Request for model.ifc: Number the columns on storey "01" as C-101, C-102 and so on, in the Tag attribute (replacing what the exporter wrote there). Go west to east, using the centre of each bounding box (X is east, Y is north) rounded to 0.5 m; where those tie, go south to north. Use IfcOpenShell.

First a look at what the model holds.

```python
import ifcopenshell
import ifcopenshell.util.element
import ifcopenshell.util.placement

model = ifcopenshell.open("model.ifc")
print(model.schema)
storey = next(s for s in model.by_type("IfcBuildingStorey") if s.Name == "01")
columns = [e for e in ifcopenshell.util.element.get_decomposition(storey) if e.is_a("IfcColumn")]
for e in sorted(columns, key=lambda e: e.id()):
    origin = ifcopenshell.util.placement.get_local_placement(e.ObjectPlacement)[:3, 3]
    print(e.id(), e.Tag, e.Name, origin.round(2) + 0.0, sep=" | ")
```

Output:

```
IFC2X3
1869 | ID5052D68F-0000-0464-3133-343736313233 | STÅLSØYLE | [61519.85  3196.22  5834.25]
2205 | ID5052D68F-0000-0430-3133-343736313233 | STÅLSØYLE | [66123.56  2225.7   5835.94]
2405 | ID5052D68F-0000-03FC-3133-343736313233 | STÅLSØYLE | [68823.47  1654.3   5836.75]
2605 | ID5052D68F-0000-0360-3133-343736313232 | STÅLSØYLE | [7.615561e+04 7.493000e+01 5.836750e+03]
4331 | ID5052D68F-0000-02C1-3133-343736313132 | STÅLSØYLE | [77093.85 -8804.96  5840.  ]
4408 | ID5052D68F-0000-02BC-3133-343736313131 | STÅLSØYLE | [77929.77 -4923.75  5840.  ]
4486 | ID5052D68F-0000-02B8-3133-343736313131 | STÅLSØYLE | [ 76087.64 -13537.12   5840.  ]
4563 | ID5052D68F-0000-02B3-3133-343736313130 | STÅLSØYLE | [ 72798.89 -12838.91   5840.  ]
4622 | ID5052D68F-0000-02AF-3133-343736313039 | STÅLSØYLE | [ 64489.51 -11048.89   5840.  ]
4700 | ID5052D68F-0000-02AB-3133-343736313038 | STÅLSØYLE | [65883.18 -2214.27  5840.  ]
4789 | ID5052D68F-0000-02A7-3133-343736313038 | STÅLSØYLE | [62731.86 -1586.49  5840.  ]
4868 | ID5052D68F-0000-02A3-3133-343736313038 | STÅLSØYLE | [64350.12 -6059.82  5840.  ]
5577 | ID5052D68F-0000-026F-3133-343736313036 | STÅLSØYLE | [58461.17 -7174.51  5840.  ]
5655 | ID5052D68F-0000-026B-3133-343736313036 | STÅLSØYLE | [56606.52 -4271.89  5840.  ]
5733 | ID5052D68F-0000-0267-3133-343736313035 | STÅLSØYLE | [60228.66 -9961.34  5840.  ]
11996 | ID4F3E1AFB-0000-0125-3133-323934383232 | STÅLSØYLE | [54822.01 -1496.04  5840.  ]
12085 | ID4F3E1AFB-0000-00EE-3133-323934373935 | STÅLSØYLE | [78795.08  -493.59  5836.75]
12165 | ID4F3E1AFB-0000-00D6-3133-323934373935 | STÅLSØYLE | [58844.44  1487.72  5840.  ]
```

```python
import ifcopenshell
import ifcopenshell.geom
import ifcopenshell.util.element
import ifcopenshell.util.shape

model = ifcopenshell.open("model.ifc")
settings = ifcopenshell.geom.settings()
settings.set("use-world-coords", True)


def centre(element):
    shape = ifcopenshell.geom.create_shape(settings, element)
    return ifcopenshell.util.shape.get_bbox_centroid(shape.geometry)


storey = next(s for s in model.by_type("IfcBuildingStorey") if s.Name == "01")
columns = [e for e in ifcopenshell.util.element.get_decomposition(storey) if e.is_a("IfcColumn")]

# Insertion points can sit at a corner or the storey origin, so sort by the geometry (in metres).
centres = {e: centre(e) for e in columns}
columns.sort(key=lambda e: (round(centres[e][0] / 0.5), centres[e][1]))

for i, e in enumerate(columns, start=1):
    number = f"C-1{i:02d}"
    e.Tag = number
    print(e.id(), number)

model.write("model_rev.ifc")
```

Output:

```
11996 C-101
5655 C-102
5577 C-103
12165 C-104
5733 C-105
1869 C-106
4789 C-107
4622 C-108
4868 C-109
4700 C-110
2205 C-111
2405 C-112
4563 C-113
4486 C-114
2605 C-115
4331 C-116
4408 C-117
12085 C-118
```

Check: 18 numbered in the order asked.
